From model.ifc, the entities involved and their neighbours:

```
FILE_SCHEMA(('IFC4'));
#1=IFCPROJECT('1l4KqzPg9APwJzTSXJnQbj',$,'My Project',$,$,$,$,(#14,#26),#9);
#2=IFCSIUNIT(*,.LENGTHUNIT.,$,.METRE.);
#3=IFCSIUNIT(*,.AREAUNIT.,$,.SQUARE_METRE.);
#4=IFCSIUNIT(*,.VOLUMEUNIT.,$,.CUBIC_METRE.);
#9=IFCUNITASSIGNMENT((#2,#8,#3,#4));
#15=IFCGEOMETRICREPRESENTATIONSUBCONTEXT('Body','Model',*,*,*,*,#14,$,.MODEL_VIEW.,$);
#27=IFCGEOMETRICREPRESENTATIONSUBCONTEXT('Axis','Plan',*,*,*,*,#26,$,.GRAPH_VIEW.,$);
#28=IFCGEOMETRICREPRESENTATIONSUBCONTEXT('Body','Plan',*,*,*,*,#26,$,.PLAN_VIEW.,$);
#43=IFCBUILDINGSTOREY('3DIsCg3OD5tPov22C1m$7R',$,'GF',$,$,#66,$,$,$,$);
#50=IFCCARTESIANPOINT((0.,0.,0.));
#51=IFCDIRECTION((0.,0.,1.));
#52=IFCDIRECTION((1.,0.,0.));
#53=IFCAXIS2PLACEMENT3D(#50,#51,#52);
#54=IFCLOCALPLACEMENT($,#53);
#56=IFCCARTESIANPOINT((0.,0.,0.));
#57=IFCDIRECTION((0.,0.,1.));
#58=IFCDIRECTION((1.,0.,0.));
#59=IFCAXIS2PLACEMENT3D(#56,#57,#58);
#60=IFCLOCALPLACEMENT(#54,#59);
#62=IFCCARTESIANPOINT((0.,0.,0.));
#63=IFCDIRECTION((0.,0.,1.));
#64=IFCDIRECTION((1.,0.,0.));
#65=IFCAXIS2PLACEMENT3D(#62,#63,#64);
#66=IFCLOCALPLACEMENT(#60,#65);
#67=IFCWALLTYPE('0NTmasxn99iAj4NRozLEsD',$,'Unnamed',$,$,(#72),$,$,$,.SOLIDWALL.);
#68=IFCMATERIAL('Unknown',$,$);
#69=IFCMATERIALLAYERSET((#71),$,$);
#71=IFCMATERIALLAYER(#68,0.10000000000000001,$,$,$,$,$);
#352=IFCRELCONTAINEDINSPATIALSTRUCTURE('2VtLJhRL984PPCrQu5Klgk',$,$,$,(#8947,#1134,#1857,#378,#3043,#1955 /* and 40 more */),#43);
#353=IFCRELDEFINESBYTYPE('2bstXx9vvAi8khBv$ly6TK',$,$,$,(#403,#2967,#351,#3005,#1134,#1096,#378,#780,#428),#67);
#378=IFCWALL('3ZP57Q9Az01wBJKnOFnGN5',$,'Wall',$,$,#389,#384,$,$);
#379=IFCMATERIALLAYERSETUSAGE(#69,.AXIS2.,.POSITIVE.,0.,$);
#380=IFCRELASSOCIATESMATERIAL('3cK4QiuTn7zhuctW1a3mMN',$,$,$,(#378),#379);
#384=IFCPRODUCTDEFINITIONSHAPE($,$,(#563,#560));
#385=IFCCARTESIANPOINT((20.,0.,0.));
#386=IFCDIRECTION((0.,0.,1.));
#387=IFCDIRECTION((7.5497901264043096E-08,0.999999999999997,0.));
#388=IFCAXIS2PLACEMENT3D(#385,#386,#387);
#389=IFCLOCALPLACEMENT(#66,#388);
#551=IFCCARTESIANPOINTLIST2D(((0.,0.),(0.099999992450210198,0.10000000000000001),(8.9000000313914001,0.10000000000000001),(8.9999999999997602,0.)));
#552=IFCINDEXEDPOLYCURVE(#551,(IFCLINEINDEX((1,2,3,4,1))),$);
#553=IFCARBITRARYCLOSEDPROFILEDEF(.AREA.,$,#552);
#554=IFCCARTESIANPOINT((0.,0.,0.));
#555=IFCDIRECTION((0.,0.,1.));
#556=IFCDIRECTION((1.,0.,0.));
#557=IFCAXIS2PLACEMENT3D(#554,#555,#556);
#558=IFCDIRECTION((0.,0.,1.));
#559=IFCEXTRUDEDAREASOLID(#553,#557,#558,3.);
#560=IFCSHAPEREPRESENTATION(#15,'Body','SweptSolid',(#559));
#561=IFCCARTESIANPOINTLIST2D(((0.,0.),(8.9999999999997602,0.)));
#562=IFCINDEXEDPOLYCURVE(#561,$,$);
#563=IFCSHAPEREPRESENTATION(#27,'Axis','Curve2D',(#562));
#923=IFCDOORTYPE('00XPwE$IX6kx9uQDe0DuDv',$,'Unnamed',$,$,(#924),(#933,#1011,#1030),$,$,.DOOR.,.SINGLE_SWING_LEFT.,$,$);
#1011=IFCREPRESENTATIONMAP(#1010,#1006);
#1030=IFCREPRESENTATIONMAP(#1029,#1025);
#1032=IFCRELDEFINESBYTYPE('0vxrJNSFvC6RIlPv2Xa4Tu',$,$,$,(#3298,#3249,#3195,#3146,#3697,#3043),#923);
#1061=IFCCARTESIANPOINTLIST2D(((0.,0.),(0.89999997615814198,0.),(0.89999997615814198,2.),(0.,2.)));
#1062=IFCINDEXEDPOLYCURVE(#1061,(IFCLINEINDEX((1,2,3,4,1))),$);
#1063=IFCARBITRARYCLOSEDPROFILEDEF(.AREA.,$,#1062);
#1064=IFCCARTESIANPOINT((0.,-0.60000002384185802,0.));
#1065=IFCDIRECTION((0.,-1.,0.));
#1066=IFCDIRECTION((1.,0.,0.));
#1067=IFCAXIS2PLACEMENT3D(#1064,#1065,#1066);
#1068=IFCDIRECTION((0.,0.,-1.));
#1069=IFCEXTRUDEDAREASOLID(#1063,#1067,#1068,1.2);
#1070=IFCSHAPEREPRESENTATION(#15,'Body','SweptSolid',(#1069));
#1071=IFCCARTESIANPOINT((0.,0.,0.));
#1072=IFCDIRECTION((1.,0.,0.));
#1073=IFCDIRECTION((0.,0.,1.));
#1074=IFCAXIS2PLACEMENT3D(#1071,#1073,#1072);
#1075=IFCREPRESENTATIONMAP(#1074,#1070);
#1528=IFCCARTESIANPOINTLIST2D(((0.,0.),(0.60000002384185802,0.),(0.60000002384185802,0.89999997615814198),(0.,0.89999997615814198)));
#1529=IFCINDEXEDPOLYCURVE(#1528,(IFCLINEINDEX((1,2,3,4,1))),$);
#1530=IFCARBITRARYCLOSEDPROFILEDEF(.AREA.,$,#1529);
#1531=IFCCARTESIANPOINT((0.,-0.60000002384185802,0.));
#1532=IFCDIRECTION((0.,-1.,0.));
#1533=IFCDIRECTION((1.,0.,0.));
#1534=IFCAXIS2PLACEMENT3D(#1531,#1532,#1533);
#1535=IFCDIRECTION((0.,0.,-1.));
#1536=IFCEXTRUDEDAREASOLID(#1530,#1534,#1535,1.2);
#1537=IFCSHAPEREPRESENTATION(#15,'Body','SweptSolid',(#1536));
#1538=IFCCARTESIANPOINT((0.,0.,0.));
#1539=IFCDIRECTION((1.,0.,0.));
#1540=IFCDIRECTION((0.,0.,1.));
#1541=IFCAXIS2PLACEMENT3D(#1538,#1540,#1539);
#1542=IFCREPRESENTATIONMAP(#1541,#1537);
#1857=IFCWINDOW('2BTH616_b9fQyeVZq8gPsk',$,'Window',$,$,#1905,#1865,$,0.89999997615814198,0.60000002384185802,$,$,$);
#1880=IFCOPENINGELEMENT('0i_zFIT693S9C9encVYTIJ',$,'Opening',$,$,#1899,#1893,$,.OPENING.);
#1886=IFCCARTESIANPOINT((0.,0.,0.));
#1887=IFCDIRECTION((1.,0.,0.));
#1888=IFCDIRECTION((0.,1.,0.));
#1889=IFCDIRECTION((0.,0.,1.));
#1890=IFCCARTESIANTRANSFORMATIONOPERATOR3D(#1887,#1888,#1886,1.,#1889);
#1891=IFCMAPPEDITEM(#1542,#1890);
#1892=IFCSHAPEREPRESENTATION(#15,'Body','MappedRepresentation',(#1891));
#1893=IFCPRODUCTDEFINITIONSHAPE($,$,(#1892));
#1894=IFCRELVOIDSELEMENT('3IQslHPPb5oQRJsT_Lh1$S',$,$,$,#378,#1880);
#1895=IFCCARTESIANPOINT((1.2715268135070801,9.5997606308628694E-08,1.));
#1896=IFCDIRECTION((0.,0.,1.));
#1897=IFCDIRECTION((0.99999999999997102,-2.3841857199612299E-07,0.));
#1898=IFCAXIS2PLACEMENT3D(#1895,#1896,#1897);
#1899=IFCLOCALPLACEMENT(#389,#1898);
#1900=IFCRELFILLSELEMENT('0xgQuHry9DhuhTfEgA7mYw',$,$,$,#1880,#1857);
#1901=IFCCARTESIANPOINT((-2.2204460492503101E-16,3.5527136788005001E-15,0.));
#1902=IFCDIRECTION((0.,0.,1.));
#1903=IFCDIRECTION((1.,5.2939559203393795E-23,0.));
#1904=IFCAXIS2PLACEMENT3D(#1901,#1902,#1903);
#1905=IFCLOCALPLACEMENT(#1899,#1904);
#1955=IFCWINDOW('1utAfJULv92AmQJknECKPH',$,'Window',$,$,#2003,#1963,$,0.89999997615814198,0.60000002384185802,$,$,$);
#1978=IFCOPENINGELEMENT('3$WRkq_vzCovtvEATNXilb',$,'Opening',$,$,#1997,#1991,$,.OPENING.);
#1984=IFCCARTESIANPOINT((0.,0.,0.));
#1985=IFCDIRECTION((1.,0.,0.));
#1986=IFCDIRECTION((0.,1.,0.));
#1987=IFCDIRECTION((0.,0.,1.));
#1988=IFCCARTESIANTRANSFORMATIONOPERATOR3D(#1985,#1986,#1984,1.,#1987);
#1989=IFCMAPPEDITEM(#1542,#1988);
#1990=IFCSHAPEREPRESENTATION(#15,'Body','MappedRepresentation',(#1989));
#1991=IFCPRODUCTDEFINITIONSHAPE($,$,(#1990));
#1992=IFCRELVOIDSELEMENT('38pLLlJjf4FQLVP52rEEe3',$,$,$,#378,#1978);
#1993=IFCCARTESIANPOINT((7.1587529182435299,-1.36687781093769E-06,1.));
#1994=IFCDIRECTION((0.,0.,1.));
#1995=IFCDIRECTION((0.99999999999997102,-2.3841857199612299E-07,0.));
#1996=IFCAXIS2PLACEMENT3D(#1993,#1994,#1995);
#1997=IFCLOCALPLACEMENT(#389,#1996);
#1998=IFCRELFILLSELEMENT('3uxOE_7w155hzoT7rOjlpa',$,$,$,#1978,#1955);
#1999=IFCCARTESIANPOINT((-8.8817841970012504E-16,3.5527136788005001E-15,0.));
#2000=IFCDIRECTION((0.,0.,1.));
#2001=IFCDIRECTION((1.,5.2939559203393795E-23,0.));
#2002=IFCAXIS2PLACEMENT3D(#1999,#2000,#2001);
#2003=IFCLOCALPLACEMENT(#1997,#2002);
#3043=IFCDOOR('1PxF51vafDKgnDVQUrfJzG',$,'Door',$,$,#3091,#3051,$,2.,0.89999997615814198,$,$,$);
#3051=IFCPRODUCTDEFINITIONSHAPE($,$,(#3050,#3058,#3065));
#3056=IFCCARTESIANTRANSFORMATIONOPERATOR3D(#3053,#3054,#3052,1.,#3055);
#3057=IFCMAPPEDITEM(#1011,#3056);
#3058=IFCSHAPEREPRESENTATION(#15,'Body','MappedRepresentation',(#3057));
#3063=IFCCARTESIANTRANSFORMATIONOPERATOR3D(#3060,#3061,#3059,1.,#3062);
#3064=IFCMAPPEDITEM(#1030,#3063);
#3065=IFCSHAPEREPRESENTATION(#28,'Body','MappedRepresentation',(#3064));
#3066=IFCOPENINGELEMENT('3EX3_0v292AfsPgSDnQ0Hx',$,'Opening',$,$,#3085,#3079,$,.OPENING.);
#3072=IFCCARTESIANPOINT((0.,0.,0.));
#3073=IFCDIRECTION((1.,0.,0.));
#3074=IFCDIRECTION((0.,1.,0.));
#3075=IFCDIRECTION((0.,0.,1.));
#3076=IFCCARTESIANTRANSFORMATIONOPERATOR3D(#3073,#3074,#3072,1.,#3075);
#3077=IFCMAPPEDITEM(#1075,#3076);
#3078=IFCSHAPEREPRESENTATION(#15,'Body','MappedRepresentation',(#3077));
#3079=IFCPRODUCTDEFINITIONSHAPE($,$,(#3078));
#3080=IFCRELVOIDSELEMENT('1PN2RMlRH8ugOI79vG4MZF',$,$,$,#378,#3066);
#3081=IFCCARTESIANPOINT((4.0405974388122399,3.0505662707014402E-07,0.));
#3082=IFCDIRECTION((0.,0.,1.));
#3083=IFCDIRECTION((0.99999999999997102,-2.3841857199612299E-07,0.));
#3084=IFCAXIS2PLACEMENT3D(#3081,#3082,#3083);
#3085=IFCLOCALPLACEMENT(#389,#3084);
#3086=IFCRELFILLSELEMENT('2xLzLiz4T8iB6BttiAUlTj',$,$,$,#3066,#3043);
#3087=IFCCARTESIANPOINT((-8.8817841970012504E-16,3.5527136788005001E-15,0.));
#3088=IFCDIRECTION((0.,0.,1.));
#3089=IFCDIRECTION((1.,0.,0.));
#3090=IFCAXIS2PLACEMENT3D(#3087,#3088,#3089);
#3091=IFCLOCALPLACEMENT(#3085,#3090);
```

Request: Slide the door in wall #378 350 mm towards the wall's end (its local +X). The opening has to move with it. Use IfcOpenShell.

```python
import ifcopenshell
import ifcopenshell.api.geometry
import ifcopenshell.util.placement
import ifcopenshell.util.unit

model = ifcopenshell.open("model.ifc")
unit_scale = ifcopenshell.util.unit.calculate_unit_scale(model)

door = model.by_guid("1PxF51vafDKgnDVQUrfJzG")
opening = door.FillsVoids[0].RelatingOpeningElement
wall = opening.VoidsElements[0].RelatingBuildingElement

wall_matrix = ifcopenshell.util.placement.get_local_placement(wall.ObjectPlacement)
shift = wall_matrix[:3, 0] * 0.35 / unit_scale
before = ifcopenshell.util.placement.get_local_placement(door.ObjectPlacement)[:3, 3].copy()

# The door is placed relative to its opening, so it follows when the opening moves.
matrix = ifcopenshell.util.placement.get_local_placement(opening.ObjectPlacement)
matrix[:3, 3] += shift
ifcopenshell.api.geometry.edit_object_placement(
    model, product=opening, matrix=matrix, is_si=False, should_transform_children=True
)

after = ifcopenshell.util.placement.get_local_placement(door.ObjectPlacement)[:3, 3]
print("door moved by", (after - before).round(3) + 0.0)

model.write("model_v2.ifc")
```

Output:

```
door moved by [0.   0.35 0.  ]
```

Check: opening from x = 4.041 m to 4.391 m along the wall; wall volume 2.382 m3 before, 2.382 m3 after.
